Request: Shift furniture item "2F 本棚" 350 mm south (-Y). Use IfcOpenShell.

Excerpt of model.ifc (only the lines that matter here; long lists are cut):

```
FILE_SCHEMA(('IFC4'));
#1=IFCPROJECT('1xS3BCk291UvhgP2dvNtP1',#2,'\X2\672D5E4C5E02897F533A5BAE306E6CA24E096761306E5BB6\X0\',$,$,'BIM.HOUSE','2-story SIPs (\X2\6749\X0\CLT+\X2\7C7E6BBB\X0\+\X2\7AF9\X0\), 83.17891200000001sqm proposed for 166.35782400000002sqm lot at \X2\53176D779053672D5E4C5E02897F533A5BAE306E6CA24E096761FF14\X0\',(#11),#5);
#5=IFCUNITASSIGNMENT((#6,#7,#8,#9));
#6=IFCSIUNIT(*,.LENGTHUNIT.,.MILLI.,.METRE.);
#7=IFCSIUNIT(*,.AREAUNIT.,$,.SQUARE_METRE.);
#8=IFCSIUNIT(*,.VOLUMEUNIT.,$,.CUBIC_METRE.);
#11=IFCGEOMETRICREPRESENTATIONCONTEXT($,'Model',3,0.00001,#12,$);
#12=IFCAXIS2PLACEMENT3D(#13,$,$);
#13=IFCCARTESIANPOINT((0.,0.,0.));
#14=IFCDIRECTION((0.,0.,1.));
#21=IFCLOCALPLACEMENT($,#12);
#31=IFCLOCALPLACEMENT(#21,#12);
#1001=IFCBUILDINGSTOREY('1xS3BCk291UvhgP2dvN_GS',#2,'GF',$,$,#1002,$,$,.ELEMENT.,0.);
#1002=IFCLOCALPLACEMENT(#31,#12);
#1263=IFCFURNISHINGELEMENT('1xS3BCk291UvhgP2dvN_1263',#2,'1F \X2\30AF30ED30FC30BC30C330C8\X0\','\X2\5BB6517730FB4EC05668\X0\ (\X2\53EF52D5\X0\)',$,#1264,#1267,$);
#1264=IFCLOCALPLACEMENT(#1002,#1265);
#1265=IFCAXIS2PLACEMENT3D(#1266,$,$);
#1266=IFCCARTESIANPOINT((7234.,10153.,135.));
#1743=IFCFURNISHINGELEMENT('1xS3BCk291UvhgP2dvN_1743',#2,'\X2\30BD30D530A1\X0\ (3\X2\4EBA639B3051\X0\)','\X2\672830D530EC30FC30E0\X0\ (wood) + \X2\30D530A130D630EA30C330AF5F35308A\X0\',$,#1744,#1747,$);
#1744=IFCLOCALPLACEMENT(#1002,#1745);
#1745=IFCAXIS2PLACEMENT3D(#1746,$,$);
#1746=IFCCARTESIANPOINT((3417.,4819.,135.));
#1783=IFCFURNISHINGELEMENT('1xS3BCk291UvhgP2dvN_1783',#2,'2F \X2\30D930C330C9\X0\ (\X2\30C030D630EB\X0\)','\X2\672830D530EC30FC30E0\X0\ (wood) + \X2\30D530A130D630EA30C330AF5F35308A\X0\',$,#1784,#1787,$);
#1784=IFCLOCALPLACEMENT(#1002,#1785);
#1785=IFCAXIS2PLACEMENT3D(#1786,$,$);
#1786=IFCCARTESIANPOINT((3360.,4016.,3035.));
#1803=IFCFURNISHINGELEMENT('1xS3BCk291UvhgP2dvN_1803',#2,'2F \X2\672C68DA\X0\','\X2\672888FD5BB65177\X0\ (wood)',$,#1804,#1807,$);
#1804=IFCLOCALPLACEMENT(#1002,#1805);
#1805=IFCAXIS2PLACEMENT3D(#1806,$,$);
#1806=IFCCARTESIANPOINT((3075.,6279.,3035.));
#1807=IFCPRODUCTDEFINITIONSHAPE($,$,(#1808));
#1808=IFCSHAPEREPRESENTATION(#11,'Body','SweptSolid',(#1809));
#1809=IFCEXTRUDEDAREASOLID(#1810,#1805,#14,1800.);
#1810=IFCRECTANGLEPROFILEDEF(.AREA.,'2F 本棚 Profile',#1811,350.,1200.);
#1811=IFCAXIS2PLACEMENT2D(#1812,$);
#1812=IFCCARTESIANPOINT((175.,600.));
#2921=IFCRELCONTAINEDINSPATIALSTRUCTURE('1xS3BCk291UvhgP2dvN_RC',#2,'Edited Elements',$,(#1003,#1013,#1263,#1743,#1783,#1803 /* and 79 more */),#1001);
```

```python
import ifcopenshell
import ifcopenshell.api.geometry
import ifcopenshell.util.placement

model = ifcopenshell.open("model.ifc")

item = model.by_guid("1xS3BCk291UvhgP2dvN_1803")
matrix = ifcopenshell.util.placement.get_local_placement(item.ObjectPlacement)
matrix[1, 3] -= 350.0
ifcopenshell.api.geometry.edit_object_placement(model, product=item, matrix=matrix, is_si=False)

print(ifcopenshell.util.placement.get_local_placement(item.ObjectPlacement).round(3) + 0.0)

model.write("model_rev.ifc")
```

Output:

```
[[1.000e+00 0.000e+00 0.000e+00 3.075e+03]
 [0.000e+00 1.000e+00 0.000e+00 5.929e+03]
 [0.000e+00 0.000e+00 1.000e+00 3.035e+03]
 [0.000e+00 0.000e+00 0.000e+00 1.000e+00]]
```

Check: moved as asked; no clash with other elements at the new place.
